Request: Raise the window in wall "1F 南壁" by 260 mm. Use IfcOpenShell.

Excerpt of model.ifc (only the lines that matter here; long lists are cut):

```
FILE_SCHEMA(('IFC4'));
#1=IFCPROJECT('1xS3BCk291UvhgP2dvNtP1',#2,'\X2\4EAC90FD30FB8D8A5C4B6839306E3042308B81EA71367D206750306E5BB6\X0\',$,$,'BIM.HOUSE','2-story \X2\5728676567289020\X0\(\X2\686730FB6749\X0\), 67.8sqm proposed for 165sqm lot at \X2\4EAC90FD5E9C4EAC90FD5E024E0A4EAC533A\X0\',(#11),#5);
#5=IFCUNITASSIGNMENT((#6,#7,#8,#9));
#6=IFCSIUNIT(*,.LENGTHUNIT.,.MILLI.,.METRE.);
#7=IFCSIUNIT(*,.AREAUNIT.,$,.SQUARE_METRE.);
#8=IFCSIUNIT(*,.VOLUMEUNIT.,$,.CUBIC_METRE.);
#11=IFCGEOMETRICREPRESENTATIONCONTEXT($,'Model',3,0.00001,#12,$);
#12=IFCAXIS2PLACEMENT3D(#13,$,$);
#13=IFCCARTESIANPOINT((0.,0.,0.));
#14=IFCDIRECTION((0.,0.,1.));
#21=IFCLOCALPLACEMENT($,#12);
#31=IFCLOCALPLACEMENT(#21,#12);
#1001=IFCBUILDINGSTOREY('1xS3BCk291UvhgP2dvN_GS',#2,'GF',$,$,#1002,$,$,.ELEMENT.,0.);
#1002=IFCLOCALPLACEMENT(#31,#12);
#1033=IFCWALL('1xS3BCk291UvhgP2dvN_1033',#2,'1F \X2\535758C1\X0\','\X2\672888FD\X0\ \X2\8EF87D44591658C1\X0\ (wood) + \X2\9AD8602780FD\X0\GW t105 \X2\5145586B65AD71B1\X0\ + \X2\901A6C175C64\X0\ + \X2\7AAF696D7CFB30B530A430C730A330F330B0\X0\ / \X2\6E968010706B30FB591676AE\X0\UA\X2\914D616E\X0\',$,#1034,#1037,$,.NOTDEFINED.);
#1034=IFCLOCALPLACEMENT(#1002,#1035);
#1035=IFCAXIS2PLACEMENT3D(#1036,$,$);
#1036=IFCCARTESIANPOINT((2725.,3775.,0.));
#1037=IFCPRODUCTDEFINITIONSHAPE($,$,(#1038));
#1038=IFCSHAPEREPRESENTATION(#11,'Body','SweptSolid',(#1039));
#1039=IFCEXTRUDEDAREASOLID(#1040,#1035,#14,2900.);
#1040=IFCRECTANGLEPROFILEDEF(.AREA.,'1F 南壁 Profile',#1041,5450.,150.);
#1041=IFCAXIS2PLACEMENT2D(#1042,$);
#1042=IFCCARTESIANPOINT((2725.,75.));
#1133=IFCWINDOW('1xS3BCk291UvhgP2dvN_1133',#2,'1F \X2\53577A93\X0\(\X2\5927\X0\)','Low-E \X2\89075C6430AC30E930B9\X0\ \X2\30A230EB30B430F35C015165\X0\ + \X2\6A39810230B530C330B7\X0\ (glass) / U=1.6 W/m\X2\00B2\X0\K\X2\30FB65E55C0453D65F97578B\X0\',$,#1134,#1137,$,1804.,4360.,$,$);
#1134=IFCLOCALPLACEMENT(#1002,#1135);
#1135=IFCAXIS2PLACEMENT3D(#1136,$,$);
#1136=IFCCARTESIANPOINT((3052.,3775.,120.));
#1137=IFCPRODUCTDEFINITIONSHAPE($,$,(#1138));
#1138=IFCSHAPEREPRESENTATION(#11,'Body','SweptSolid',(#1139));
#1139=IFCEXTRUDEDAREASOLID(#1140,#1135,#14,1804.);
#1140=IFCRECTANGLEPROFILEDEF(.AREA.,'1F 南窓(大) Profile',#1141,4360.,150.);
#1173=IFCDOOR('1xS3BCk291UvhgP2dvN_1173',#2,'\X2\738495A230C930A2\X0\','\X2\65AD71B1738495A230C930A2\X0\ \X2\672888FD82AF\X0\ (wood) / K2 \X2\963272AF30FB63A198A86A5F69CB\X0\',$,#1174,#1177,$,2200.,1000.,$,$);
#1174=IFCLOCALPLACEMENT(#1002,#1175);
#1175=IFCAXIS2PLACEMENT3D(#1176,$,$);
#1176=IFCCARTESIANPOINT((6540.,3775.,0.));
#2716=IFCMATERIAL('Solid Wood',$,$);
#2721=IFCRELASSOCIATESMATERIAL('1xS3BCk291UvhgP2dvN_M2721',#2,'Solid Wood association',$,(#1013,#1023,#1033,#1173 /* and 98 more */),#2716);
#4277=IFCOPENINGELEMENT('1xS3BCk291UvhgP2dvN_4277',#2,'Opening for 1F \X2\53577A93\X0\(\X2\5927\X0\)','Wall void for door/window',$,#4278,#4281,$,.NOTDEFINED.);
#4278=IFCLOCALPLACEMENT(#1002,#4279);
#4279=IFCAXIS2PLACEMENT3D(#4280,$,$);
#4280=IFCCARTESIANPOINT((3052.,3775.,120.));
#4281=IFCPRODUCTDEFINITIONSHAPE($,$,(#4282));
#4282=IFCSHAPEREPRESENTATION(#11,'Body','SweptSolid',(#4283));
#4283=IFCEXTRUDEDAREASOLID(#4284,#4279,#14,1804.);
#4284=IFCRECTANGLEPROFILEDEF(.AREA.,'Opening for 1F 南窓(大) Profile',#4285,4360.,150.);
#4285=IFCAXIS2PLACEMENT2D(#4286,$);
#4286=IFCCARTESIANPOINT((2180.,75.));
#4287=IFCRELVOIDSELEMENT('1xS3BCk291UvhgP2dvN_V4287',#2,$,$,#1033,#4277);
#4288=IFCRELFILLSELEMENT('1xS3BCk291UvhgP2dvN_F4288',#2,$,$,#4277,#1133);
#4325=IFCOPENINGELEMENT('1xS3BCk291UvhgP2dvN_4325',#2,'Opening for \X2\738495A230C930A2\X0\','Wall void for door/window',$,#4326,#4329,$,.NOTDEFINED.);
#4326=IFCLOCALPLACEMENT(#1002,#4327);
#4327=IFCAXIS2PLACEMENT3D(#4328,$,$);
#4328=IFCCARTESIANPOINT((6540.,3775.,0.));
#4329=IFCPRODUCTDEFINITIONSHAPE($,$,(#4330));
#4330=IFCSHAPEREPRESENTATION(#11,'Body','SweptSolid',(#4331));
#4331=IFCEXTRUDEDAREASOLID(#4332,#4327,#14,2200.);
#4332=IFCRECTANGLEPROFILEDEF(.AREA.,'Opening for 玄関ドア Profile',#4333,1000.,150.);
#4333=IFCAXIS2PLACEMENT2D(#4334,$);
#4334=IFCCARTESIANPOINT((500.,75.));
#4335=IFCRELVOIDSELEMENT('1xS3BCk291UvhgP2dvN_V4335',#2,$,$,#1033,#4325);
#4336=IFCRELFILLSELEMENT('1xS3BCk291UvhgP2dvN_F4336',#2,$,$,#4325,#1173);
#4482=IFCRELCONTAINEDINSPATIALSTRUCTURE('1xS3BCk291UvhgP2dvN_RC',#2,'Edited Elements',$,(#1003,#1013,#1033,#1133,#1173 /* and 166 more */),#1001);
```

```python
import numpy as np
import ifcopenshell
import ifcopenshell.api.geometry
import ifcopenshell.util.placement
import ifcopenshell.util.unit

model = ifcopenshell.open("model.ifc")
unit_scale = ifcopenshell.util.unit.calculate_unit_scale(model)

window = model.by_guid("1xS3BCk291UvhgP2dvN_1133")
opening = window.FillsVoids[0].RelatingOpeningElement
dz = 0.26 / unit_scale

shift = np.array([0.0, 0.0, dz])
# The window is not placed relative to its opening, so move both.
for product in (opening, window):
    matrix = ifcopenshell.util.placement.get_local_placement(product.ObjectPlacement)
    matrix[:3, 3] += shift
    ifcopenshell.api.geometry.edit_object_placement(model, product=product, matrix=matrix, is_si=False)

print(f"moved by {dz * unit_scale:+.3f} m")

model.write("model_v2.ifc")
```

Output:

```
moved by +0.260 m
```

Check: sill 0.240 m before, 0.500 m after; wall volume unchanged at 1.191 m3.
